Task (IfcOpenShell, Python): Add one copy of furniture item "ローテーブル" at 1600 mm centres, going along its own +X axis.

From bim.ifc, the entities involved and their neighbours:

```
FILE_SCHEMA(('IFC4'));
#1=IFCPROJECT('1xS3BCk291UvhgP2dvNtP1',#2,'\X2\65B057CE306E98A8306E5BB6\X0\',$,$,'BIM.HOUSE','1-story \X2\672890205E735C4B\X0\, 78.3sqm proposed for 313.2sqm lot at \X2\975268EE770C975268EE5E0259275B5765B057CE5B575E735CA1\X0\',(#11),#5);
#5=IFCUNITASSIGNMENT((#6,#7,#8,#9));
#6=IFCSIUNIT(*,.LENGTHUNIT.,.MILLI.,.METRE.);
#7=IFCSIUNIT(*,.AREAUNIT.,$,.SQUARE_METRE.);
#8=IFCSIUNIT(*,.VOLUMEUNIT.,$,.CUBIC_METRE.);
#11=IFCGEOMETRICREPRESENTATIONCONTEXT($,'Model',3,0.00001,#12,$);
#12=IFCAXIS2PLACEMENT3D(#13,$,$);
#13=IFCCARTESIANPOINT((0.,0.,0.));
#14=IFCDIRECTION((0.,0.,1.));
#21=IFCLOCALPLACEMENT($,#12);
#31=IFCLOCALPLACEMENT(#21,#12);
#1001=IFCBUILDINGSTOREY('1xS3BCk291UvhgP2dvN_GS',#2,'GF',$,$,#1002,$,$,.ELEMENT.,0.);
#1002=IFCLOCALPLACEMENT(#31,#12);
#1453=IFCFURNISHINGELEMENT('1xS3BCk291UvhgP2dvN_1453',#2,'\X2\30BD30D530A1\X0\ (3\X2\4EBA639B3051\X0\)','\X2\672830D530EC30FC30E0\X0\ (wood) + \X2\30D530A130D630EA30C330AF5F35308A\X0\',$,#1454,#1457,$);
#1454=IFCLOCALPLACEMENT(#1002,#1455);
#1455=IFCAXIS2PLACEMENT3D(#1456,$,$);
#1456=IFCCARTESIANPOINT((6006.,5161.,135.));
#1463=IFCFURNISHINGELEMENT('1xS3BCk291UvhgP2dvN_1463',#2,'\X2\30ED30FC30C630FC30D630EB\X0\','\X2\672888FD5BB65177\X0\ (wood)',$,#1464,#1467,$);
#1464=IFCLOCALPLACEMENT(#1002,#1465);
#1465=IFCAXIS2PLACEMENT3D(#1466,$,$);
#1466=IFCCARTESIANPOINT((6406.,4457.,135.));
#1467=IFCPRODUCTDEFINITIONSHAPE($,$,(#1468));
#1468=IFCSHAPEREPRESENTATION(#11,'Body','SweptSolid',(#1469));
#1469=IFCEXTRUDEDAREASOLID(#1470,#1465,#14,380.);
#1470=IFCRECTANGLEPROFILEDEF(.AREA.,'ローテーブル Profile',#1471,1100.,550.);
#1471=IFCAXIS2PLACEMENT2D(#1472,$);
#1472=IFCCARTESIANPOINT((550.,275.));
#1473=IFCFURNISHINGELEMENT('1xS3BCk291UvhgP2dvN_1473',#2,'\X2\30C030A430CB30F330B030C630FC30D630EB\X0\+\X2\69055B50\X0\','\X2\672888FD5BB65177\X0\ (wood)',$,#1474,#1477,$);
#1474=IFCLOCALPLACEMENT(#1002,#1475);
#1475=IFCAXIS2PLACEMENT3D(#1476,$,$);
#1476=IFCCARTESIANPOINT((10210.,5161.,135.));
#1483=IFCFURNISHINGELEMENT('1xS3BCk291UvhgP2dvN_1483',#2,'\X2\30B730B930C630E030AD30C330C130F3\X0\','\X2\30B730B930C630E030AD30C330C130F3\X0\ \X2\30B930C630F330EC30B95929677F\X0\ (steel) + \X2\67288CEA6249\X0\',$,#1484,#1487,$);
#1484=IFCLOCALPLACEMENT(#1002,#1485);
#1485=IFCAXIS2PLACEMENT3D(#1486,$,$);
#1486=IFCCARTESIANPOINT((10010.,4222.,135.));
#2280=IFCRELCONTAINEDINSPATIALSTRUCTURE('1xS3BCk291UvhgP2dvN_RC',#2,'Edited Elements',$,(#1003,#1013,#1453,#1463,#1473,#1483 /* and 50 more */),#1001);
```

```python
import ifcopenshell
import ifcopenshell.api.geometry
import ifcopenshell.api.root
import ifcopenshell.util.element
import ifcopenshell.util.placement

model = ifcopenshell.open("bim.ifc")


def reuse_history(source, copy):
    """copy_class also copies each property set's owner history, people and application; keep the originals."""
    for rel in copy.IsDefinedBy:
        if rel.is_a("IfcRelDefinesByProperties") and (history := rel.RelatingPropertyDefinition.OwnerHistory):
            rel.RelatingPropertyDefinition.OwnerHistory = source.OwnerHistory
            ifcopenshell.util.element.remove_deep2(model, history)


source = model.by_guid("1xS3BCk291UvhgP2dvN_1463")
base = ifcopenshell.util.placement.get_local_placement(source.ObjectPlacement)
step = base[:3, 0] * 1600.0

for i in range(1, 2):
    copy = ifcopenshell.api.root.copy_class(model, product=source)
    copy.Representation = ifcopenshell.util.element.copy_deep(
        model, source.Representation, exclude=["IfcGeometricRepresentationContext", "IfcRepresentationMap"]
    )
    reuse_history(source, copy)
    matrix = base.copy()
    matrix[:3, 3] += i * step
    print("added at", matrix[:3, 3].round(3) + 0.0)
    ifcopenshell.api.geometry.edit_object_placement(model, product=copy, matrix=matrix, is_si=False)

model.write("bim_v2.ifc")
```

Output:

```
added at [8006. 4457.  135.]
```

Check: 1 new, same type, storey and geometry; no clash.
